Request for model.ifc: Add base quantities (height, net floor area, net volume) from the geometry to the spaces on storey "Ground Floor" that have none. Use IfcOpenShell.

First a look at what the model holds.

```python
import ifcopenshell
import ifcopenshell.util.element
import ifcopenshell.util.unit

model = ifcopenshell.open("model.ifc")
print(model.schema)
for unit_type in ("LENGTHUNIT", "AREAUNIT", "VOLUMEUNIT"):
    print(unit_type, ifcopenshell.util.unit.calculate_unit_scale(model, unit_type))
storey = next(s for s in model.by_type("IfcBuildingStorey") if s.Name == "Ground Floor")
spaces = [e for e in ifcopenshell.util.element.get_decomposition(storey) if e.is_a("IfcSpace")]
for e in sorted(spaces, key=lambda e: e.id()):
    print(e.id(), e.is_a(), e.Name, list(ifcopenshell.util.element.get_psets(e, qtos_only=True)), sep=" | ")
```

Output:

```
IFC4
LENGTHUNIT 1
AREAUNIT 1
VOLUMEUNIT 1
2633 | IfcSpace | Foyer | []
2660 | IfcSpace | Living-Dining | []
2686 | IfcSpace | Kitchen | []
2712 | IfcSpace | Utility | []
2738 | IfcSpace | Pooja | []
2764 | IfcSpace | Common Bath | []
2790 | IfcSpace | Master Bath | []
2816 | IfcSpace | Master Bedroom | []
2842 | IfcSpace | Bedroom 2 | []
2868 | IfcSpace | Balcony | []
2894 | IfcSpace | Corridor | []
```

```python
import ifcopenshell
import ifcopenshell.api.pset
import ifcopenshell.geom
import ifcopenshell.util.element
import ifcopenshell.util.shape
import ifcopenshell.util.unit

model = ifcopenshell.open("model.ifc")
unit_scale = ifcopenshell.util.unit.calculate_unit_scale(model)
area_scale = ifcopenshell.util.unit.calculate_unit_scale(model, "AREAUNIT")
volume_scale = ifcopenshell.util.unit.calculate_unit_scale(model, "VOLUMEUNIT")
settings = ifcopenshell.geom.settings()

storey = next(s for s in model.by_type("IfcBuildingStorey") if s.Name == "Ground Floor")
spaces = [e for e in ifcopenshell.util.element.get_decomposition(storey) if e.is_a("IfcSpace")]

for e in sorted(spaces, key=lambda e: e.id()):
    if ifcopenshell.util.element.get_psets(e, qtos_only=True, should_inherit=False):
        continue
    # Geometry comes back in metres, in the element's own axes.
    shape = ifcopenshell.geom.create_shape(settings, e)
    values = {
        "Height": ifcopenshell.util.shape.get_z(shape.geometry) / unit_scale,
        "NetFloorArea": ifcopenshell.util.shape.get_footprint_area(shape.geometry) / area_scale,
        "NetVolume": ifcopenshell.util.shape.get_volume(shape.geometry) / volume_scale,
    }
    qto = ifcopenshell.api.pset.add_qto(model, product=e, name="Qto_SpaceBaseQuantities")
    ifcopenshell.api.pset.edit_qto(model, qto=qto, properties=values)
    print(e.id(), {k: round(v, 3) for k, v in values.items()})

model.write("model_updated.ifc")
```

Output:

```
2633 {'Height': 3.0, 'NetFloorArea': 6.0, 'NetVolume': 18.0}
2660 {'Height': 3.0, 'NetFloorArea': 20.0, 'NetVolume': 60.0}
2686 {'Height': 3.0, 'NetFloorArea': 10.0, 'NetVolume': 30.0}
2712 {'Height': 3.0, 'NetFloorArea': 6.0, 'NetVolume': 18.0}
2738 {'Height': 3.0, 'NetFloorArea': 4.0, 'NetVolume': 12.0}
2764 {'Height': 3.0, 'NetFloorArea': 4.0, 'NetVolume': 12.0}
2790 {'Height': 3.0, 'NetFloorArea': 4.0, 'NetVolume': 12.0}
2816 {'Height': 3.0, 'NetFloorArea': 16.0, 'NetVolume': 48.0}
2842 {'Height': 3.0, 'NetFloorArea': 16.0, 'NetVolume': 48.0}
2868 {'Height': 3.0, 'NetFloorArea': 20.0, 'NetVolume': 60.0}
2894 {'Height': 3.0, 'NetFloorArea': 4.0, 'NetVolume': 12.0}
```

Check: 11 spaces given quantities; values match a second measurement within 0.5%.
